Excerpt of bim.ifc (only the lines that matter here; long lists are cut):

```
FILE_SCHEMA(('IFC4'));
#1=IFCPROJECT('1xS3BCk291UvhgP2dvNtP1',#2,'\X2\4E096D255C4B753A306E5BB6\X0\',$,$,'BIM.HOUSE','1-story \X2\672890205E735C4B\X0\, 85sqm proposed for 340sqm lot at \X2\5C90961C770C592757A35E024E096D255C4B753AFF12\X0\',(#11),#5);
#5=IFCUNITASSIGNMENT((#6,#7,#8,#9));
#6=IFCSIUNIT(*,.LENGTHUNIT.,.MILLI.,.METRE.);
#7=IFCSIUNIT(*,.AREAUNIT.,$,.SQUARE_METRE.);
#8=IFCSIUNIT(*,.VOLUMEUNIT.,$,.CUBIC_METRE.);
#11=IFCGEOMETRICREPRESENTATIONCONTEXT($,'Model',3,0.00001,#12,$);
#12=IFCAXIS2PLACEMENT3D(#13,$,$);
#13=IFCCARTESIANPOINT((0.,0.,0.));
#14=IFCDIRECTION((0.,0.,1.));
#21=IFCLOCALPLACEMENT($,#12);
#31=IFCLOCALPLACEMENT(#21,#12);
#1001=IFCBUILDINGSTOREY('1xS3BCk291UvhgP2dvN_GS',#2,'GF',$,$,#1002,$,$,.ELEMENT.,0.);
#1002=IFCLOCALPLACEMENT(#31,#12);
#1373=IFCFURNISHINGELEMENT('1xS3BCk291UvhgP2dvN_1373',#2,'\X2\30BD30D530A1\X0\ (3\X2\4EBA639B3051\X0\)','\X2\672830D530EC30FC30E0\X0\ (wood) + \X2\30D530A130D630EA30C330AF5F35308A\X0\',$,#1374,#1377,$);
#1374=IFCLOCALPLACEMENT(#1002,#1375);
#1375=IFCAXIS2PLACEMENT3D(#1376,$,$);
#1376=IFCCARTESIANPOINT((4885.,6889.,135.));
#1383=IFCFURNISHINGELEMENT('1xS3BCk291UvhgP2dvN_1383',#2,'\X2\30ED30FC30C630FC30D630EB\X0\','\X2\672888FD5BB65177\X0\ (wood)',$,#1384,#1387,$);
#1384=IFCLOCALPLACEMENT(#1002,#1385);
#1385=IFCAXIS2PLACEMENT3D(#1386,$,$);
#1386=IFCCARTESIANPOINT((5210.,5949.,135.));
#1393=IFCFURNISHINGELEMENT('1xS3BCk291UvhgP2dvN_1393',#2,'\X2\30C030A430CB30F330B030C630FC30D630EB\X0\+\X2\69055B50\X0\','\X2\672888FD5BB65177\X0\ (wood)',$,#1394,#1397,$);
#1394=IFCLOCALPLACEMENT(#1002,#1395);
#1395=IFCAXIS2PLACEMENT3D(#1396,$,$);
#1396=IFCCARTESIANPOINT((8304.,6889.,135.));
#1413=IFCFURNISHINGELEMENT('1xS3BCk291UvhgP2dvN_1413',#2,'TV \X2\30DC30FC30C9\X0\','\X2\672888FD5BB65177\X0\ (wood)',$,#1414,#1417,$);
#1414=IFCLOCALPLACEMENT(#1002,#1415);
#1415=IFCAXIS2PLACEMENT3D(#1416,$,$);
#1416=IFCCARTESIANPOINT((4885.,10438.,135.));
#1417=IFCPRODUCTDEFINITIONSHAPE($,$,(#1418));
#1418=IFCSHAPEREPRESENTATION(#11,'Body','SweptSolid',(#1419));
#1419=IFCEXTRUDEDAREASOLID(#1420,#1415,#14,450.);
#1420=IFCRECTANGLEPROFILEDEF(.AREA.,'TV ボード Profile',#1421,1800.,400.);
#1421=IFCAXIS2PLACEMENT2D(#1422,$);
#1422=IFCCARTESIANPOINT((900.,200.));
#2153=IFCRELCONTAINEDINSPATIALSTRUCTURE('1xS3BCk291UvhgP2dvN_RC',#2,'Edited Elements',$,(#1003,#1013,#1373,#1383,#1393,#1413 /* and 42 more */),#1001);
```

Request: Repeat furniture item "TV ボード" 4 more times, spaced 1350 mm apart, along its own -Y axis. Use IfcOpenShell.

```python
import ifcopenshell
import ifcopenshell.api.geometry
import ifcopenshell.api.root
import ifcopenshell.util.element
import ifcopenshell.util.placement

model = ifcopenshell.open("bim.ifc")


def reuse_history(source, copy):
    """copy_class also copies each property set's owner history, people and application; keep the originals."""
    for rel in copy.IsDefinedBy:
        if rel.is_a("IfcRelDefinesByProperties") and (history := rel.RelatingPropertyDefinition.OwnerHistory):
            rel.RelatingPropertyDefinition.OwnerHistory = source.OwnerHistory
            ifcopenshell.util.element.remove_deep2(model, history)


source = model.by_id(1413)
base = ifcopenshell.util.placement.get_local_placement(source.ObjectPlacement)
step = -base[:3, 1] * 1350.0

for i in range(1, 5):
    copy = ifcopenshell.api.root.copy_class(model, product=source)
    copy.Representation = ifcopenshell.util.element.copy_deep(
        model, source.Representation, exclude=["IfcGeometricRepresentationContext", "IfcRepresentationMap"]
    )
    reuse_history(source, copy)
    matrix = base.copy()
    matrix[:3, 3] += i * step
    print("added at", matrix[:3, 3].round(3) + 0.0)
    ifcopenshell.api.geometry.edit_object_placement(model, product=copy, matrix=matrix, is_si=False)

model.write("bim_v2.ifc")
```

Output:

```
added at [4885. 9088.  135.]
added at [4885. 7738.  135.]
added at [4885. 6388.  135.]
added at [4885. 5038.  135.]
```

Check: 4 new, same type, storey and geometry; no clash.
